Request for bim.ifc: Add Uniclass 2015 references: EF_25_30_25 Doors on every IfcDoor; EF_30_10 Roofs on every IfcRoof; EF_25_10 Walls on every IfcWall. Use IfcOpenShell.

First a look at what the model holds.

```python
import ifcopenshell

model = ifcopenshell.open("bim.ifc")
print(model.schema)
print("classifications:", [c.Name for c in model.by_type("IfcClassification")])
for ifc_class in ("IfcDoor", "IfcRoof", "IfcStair", "IfcWall", "IfcWindow"):
    print(ifc_class, len(model.by_type(ifc_class)))
```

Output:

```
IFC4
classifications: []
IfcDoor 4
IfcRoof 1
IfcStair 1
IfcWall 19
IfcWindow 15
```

```python
import ifcopenshell
import ifcopenshell.api.classification

model = ifcopenshell.open("bim.ifc")

system = ifcopenshell.api.classification.add_classification(model, classification="Uniclass 2015")

codes = {
    "IfcDoor": ("EF_25_30_25", "Doors"),
    "IfcRoof": ("EF_30_10", "Roofs"),
    "IfcWall": ("EF_25_10", "Walls"),
}
for ifc_class, (code, name) in codes.items():
    products = model.by_type(ifc_class)
    ifcopenshell.api.classification.add_reference(
        model, products=products, classification=system, identification=code, name=name
    )
    print(code, len(products))

model.write("bim_rev.ifc")
```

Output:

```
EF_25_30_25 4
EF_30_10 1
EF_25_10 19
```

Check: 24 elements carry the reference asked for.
